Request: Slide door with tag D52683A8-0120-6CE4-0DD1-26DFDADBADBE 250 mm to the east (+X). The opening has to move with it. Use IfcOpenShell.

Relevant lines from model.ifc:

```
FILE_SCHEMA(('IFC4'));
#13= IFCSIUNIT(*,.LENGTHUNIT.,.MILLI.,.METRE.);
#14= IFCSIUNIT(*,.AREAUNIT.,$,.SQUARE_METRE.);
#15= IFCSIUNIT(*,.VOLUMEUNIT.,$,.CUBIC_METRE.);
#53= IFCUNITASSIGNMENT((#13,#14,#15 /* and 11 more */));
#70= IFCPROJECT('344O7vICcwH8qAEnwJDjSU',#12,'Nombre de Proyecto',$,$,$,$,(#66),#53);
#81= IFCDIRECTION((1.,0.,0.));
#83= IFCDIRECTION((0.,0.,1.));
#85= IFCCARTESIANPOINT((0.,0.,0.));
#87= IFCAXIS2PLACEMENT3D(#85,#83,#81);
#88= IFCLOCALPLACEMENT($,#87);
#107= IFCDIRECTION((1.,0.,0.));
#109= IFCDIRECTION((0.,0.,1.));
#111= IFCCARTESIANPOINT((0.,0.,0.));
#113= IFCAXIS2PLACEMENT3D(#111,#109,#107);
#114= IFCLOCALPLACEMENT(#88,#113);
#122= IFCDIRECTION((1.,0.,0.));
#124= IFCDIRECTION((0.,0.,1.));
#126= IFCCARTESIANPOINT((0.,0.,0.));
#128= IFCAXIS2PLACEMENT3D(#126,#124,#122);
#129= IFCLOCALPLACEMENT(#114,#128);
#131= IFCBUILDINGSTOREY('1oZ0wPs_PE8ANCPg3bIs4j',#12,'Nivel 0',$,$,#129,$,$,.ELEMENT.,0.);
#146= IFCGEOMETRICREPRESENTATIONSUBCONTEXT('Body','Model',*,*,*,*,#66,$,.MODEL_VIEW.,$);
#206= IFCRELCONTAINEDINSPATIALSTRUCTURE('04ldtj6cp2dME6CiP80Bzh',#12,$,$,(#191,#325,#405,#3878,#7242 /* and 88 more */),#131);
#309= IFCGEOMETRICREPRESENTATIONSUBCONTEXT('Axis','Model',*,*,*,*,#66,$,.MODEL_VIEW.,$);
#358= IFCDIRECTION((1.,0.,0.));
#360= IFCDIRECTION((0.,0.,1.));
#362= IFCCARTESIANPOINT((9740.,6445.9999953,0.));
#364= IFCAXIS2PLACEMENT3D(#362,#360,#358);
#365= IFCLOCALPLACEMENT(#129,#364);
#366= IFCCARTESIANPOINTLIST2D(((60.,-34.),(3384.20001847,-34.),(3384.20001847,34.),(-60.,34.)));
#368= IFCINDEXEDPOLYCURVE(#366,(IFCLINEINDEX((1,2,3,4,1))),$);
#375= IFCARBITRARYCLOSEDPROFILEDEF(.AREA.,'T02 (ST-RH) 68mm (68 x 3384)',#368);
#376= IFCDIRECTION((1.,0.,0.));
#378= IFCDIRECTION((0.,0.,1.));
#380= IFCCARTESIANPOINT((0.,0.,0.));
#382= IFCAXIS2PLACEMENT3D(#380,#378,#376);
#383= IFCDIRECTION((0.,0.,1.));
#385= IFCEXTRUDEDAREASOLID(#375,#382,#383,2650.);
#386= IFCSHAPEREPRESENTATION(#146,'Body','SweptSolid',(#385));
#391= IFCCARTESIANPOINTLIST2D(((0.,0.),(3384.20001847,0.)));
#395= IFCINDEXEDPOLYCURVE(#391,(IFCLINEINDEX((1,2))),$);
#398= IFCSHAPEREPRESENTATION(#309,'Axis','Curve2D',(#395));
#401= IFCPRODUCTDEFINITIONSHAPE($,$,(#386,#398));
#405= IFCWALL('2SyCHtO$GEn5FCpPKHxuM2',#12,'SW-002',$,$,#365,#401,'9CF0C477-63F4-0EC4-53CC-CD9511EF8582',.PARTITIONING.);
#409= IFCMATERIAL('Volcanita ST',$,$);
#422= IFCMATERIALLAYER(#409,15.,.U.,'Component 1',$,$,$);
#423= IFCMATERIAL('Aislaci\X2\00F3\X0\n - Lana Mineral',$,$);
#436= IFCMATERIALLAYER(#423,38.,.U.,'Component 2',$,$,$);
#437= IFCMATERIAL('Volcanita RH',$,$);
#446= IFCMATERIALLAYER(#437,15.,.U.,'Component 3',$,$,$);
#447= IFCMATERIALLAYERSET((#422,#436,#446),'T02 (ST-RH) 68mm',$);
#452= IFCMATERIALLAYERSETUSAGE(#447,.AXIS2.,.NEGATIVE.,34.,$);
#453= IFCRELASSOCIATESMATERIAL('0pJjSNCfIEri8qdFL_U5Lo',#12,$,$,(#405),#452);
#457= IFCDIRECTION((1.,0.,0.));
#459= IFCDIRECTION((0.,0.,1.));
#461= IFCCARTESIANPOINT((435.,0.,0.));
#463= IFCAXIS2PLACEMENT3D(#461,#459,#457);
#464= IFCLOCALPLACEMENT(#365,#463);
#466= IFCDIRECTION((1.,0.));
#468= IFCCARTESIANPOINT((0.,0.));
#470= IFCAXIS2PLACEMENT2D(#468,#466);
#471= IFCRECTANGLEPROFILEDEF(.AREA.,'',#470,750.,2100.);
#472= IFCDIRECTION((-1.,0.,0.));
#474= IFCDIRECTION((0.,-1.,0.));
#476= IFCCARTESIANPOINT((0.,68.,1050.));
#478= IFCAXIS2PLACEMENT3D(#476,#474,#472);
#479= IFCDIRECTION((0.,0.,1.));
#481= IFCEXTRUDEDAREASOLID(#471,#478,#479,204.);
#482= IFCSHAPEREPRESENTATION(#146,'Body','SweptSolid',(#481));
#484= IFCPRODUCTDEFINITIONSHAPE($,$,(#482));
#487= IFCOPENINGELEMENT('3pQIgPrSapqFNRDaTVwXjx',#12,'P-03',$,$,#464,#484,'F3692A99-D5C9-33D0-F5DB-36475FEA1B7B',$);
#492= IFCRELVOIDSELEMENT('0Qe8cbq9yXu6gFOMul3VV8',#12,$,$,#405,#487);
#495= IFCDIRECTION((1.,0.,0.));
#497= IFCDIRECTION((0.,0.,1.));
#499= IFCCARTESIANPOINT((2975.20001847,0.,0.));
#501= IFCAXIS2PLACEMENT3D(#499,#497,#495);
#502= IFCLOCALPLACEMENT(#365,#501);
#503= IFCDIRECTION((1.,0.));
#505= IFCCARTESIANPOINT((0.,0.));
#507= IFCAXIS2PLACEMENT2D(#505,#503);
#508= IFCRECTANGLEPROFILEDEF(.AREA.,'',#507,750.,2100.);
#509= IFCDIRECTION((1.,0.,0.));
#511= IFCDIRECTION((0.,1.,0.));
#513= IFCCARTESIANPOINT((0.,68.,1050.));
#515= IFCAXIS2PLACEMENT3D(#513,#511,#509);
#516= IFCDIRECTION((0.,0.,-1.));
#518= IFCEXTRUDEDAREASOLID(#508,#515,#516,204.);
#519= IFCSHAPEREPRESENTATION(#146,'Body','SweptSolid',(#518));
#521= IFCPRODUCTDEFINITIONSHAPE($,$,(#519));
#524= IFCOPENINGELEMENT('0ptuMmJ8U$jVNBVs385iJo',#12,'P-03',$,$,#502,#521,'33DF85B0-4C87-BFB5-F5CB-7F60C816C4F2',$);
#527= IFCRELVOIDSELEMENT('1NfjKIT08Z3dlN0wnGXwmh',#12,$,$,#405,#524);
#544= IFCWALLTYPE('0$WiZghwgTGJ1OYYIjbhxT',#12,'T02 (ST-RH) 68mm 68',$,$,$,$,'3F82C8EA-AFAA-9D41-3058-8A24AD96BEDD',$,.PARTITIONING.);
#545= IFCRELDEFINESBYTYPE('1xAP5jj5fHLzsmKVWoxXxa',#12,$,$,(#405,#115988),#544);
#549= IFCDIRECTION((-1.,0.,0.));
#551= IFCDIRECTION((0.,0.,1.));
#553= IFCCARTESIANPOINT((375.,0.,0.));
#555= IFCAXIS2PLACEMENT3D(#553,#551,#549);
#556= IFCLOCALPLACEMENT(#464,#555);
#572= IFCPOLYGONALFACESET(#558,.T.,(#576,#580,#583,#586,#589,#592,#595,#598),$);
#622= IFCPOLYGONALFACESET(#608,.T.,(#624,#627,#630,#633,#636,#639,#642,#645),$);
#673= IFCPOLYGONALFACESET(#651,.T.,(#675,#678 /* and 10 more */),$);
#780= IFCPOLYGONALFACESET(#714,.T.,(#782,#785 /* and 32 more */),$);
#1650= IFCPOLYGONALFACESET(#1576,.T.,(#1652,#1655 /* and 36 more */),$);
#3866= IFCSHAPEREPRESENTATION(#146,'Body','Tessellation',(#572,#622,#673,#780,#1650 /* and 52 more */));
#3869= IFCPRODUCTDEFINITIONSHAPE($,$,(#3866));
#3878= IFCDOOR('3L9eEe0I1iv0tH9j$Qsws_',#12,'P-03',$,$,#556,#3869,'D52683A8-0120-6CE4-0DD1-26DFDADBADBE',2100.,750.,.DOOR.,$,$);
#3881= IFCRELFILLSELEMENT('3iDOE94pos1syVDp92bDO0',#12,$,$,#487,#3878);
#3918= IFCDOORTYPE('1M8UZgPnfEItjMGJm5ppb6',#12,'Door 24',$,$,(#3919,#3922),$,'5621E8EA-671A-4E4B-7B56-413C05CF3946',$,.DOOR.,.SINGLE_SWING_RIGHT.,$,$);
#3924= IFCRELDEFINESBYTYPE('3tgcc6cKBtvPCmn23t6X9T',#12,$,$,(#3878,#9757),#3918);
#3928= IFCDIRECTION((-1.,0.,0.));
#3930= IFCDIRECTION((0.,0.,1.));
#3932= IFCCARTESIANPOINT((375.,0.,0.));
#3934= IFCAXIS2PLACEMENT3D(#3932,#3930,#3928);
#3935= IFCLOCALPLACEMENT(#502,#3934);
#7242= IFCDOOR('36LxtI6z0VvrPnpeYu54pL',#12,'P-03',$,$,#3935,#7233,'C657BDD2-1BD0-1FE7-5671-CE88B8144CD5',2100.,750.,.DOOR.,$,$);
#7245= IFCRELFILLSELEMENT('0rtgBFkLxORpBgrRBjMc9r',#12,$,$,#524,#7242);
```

```python
import ifcopenshell
import ifcopenshell.api.geometry
import ifcopenshell.util.placement
import ifcopenshell.util.unit

model = ifcopenshell.open("model.ifc")
unit_scale = ifcopenshell.util.unit.calculate_unit_scale(model)

door = model.by_guid("3L9eEe0I1iv0tH9j$Qsws_")
opening = door.FillsVoids[0].RelatingOpeningElement
wall = opening.VoidsElements[0].RelatingBuildingElement

wall_matrix = ifcopenshell.util.placement.get_local_placement(wall.ObjectPlacement)
shift = wall_matrix[:3, 0] * 0.25 / unit_scale
before = ifcopenshell.util.placement.get_local_placement(door.ObjectPlacement)[:3, 3].copy()

# The door is placed relative to its opening, so it follows when the opening moves.
matrix = ifcopenshell.util.placement.get_local_placement(opening.ObjectPlacement)
matrix[:3, 3] += shift
ifcopenshell.api.geometry.edit_object_placement(
    model, product=opening, matrix=matrix, is_si=False, should_transform_children=True
)

after = ifcopenshell.util.placement.get_local_placement(door.ObjectPlacement)[:3, 3]
print("door moved by", (after - before).round(3) + 0.0)

model.write("model_v2.ifc")
```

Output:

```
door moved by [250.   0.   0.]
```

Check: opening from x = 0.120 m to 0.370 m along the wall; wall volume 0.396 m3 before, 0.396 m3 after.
